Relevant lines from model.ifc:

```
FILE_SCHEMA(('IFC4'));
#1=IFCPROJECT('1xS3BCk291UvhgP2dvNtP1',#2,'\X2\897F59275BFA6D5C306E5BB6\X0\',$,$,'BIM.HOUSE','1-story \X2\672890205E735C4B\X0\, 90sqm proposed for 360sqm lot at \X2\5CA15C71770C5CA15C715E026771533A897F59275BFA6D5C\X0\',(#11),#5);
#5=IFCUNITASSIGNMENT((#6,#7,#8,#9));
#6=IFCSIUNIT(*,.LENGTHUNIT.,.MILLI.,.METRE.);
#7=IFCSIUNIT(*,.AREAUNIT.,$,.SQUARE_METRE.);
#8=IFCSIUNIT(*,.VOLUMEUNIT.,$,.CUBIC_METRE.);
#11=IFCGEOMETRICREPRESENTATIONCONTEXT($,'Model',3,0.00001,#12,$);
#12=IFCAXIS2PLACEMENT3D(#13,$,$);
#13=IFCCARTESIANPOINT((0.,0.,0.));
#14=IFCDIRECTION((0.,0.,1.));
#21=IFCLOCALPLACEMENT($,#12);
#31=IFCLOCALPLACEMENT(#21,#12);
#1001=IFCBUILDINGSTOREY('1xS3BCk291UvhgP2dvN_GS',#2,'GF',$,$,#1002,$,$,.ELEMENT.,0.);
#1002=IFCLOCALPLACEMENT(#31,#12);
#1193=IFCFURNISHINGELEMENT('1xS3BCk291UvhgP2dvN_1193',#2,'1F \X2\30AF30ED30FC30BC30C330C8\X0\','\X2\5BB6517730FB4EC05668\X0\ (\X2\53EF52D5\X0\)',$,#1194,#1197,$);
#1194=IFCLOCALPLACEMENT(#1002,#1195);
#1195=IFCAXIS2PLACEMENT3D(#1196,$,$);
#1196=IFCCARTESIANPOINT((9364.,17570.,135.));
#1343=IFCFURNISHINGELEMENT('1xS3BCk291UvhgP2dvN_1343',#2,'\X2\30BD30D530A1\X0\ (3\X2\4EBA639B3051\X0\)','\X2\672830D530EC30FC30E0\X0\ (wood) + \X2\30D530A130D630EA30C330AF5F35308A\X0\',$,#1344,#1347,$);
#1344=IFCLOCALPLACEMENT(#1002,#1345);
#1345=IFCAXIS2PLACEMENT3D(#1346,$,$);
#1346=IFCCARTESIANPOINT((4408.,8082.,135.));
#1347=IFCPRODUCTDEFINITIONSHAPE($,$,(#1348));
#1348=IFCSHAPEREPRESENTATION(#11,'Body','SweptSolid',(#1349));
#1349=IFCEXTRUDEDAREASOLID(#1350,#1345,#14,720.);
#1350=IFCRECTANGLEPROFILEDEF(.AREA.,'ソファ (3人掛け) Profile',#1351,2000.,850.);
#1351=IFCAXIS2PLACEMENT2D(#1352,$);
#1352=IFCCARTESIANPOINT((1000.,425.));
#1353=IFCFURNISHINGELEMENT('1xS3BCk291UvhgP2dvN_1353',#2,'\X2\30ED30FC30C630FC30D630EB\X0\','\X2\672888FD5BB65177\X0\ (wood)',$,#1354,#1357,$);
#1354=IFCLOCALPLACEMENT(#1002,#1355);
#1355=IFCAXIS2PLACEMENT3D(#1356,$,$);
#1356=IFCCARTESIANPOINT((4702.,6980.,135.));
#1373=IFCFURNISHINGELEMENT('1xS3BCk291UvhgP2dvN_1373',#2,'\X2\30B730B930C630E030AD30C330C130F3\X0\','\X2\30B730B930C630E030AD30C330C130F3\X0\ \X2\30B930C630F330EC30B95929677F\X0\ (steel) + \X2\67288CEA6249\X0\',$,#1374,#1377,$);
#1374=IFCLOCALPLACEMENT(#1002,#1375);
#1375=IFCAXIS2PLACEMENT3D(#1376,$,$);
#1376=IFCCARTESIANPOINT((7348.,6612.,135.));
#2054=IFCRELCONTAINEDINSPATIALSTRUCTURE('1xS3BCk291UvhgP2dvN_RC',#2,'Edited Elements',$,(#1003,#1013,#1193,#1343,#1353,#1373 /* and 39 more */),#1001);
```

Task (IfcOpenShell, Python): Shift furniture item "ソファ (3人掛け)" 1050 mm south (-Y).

```python
import ifcopenshell
import ifcopenshell.api.geometry
import ifcopenshell.util.placement
import ifcopenshell.util.unit

model = ifcopenshell.open("model.ifc")
unit_scale = ifcopenshell.util.unit.calculate_unit_scale(model)

item = model.by_guid("1xS3BCk291UvhgP2dvN_1343")
matrix = ifcopenshell.util.placement.get_local_placement(item.ObjectPlacement)
matrix[1, 3] -= 1.05 / unit_scale
ifcopenshell.api.geometry.edit_object_placement(model, product=item, matrix=matrix, is_si=False)

print(ifcopenshell.util.placement.get_local_placement(item.ObjectPlacement).round(3) + 0.0)

model.write("model_updated.ifc")
```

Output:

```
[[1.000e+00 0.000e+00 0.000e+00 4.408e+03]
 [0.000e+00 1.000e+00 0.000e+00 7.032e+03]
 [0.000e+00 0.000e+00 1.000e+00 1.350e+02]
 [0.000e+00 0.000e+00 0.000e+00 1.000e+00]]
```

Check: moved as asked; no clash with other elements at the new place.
